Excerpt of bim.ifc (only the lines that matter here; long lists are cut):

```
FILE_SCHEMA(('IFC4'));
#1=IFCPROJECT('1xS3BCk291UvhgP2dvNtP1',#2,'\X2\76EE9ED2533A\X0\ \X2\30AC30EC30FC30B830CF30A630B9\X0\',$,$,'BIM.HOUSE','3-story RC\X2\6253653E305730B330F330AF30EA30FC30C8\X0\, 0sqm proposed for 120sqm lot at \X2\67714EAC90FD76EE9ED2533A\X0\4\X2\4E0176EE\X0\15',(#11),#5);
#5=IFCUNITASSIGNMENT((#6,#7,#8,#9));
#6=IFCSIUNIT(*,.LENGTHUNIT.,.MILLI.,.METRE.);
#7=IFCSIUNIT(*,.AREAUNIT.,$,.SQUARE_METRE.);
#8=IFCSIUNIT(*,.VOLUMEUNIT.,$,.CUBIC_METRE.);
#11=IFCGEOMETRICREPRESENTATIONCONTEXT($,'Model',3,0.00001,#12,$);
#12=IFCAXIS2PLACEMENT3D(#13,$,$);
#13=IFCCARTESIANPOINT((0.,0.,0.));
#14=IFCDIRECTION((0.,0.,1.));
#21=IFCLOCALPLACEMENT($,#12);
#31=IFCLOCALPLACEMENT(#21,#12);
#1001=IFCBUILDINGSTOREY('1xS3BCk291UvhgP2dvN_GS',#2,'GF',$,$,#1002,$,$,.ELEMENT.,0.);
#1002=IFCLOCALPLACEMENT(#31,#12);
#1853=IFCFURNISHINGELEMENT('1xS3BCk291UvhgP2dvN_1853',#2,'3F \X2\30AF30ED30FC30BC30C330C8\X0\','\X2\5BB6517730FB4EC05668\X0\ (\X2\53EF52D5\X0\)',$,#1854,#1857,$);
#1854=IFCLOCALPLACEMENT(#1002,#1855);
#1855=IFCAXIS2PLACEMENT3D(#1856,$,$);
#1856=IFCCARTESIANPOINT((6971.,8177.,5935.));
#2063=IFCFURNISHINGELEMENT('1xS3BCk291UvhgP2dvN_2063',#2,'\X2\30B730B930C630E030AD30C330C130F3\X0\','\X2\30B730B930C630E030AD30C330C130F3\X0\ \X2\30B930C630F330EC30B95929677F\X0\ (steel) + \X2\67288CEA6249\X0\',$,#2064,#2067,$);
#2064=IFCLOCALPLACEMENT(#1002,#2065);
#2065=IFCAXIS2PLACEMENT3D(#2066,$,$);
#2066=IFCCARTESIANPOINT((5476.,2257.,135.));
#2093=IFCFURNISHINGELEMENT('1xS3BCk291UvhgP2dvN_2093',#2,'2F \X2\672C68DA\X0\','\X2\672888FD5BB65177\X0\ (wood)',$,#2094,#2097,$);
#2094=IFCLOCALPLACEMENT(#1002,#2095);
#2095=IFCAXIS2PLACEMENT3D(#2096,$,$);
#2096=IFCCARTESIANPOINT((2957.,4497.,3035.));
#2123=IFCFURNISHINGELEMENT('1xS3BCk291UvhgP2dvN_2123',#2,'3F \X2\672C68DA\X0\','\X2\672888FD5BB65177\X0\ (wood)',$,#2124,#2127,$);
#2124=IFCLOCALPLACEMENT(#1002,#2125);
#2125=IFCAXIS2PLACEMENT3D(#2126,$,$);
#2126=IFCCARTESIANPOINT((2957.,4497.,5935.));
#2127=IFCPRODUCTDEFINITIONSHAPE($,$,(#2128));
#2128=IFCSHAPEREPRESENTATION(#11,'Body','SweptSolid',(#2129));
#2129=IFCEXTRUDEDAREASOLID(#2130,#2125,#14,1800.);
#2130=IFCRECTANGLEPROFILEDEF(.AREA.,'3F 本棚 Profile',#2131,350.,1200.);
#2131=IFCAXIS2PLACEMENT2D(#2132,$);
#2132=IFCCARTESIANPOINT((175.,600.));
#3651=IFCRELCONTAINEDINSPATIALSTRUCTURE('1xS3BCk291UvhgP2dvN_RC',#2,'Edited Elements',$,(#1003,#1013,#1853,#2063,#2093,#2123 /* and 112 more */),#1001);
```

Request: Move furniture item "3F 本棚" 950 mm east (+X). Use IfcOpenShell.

```python
import ifcopenshell
import ifcopenshell.api.geometry
import ifcopenshell.util.placement

model = ifcopenshell.open("bim.ifc")

item = model.by_guid("1xS3BCk291UvhgP2dvN_2123")
matrix = ifcopenshell.util.placement.get_local_placement(item.ObjectPlacement)
matrix[0, 3] += 950.0
ifcopenshell.api.geometry.edit_object_placement(model, product=item, matrix=matrix, is_si=False)

print(ifcopenshell.util.placement.get_local_placement(item.ObjectPlacement).round(3) + 0.0)

model.write("bim_rev.ifc")
```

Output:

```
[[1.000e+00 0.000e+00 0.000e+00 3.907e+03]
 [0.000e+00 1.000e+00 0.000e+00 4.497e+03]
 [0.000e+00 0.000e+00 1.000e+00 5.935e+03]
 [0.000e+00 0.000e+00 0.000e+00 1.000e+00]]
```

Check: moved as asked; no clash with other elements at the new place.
